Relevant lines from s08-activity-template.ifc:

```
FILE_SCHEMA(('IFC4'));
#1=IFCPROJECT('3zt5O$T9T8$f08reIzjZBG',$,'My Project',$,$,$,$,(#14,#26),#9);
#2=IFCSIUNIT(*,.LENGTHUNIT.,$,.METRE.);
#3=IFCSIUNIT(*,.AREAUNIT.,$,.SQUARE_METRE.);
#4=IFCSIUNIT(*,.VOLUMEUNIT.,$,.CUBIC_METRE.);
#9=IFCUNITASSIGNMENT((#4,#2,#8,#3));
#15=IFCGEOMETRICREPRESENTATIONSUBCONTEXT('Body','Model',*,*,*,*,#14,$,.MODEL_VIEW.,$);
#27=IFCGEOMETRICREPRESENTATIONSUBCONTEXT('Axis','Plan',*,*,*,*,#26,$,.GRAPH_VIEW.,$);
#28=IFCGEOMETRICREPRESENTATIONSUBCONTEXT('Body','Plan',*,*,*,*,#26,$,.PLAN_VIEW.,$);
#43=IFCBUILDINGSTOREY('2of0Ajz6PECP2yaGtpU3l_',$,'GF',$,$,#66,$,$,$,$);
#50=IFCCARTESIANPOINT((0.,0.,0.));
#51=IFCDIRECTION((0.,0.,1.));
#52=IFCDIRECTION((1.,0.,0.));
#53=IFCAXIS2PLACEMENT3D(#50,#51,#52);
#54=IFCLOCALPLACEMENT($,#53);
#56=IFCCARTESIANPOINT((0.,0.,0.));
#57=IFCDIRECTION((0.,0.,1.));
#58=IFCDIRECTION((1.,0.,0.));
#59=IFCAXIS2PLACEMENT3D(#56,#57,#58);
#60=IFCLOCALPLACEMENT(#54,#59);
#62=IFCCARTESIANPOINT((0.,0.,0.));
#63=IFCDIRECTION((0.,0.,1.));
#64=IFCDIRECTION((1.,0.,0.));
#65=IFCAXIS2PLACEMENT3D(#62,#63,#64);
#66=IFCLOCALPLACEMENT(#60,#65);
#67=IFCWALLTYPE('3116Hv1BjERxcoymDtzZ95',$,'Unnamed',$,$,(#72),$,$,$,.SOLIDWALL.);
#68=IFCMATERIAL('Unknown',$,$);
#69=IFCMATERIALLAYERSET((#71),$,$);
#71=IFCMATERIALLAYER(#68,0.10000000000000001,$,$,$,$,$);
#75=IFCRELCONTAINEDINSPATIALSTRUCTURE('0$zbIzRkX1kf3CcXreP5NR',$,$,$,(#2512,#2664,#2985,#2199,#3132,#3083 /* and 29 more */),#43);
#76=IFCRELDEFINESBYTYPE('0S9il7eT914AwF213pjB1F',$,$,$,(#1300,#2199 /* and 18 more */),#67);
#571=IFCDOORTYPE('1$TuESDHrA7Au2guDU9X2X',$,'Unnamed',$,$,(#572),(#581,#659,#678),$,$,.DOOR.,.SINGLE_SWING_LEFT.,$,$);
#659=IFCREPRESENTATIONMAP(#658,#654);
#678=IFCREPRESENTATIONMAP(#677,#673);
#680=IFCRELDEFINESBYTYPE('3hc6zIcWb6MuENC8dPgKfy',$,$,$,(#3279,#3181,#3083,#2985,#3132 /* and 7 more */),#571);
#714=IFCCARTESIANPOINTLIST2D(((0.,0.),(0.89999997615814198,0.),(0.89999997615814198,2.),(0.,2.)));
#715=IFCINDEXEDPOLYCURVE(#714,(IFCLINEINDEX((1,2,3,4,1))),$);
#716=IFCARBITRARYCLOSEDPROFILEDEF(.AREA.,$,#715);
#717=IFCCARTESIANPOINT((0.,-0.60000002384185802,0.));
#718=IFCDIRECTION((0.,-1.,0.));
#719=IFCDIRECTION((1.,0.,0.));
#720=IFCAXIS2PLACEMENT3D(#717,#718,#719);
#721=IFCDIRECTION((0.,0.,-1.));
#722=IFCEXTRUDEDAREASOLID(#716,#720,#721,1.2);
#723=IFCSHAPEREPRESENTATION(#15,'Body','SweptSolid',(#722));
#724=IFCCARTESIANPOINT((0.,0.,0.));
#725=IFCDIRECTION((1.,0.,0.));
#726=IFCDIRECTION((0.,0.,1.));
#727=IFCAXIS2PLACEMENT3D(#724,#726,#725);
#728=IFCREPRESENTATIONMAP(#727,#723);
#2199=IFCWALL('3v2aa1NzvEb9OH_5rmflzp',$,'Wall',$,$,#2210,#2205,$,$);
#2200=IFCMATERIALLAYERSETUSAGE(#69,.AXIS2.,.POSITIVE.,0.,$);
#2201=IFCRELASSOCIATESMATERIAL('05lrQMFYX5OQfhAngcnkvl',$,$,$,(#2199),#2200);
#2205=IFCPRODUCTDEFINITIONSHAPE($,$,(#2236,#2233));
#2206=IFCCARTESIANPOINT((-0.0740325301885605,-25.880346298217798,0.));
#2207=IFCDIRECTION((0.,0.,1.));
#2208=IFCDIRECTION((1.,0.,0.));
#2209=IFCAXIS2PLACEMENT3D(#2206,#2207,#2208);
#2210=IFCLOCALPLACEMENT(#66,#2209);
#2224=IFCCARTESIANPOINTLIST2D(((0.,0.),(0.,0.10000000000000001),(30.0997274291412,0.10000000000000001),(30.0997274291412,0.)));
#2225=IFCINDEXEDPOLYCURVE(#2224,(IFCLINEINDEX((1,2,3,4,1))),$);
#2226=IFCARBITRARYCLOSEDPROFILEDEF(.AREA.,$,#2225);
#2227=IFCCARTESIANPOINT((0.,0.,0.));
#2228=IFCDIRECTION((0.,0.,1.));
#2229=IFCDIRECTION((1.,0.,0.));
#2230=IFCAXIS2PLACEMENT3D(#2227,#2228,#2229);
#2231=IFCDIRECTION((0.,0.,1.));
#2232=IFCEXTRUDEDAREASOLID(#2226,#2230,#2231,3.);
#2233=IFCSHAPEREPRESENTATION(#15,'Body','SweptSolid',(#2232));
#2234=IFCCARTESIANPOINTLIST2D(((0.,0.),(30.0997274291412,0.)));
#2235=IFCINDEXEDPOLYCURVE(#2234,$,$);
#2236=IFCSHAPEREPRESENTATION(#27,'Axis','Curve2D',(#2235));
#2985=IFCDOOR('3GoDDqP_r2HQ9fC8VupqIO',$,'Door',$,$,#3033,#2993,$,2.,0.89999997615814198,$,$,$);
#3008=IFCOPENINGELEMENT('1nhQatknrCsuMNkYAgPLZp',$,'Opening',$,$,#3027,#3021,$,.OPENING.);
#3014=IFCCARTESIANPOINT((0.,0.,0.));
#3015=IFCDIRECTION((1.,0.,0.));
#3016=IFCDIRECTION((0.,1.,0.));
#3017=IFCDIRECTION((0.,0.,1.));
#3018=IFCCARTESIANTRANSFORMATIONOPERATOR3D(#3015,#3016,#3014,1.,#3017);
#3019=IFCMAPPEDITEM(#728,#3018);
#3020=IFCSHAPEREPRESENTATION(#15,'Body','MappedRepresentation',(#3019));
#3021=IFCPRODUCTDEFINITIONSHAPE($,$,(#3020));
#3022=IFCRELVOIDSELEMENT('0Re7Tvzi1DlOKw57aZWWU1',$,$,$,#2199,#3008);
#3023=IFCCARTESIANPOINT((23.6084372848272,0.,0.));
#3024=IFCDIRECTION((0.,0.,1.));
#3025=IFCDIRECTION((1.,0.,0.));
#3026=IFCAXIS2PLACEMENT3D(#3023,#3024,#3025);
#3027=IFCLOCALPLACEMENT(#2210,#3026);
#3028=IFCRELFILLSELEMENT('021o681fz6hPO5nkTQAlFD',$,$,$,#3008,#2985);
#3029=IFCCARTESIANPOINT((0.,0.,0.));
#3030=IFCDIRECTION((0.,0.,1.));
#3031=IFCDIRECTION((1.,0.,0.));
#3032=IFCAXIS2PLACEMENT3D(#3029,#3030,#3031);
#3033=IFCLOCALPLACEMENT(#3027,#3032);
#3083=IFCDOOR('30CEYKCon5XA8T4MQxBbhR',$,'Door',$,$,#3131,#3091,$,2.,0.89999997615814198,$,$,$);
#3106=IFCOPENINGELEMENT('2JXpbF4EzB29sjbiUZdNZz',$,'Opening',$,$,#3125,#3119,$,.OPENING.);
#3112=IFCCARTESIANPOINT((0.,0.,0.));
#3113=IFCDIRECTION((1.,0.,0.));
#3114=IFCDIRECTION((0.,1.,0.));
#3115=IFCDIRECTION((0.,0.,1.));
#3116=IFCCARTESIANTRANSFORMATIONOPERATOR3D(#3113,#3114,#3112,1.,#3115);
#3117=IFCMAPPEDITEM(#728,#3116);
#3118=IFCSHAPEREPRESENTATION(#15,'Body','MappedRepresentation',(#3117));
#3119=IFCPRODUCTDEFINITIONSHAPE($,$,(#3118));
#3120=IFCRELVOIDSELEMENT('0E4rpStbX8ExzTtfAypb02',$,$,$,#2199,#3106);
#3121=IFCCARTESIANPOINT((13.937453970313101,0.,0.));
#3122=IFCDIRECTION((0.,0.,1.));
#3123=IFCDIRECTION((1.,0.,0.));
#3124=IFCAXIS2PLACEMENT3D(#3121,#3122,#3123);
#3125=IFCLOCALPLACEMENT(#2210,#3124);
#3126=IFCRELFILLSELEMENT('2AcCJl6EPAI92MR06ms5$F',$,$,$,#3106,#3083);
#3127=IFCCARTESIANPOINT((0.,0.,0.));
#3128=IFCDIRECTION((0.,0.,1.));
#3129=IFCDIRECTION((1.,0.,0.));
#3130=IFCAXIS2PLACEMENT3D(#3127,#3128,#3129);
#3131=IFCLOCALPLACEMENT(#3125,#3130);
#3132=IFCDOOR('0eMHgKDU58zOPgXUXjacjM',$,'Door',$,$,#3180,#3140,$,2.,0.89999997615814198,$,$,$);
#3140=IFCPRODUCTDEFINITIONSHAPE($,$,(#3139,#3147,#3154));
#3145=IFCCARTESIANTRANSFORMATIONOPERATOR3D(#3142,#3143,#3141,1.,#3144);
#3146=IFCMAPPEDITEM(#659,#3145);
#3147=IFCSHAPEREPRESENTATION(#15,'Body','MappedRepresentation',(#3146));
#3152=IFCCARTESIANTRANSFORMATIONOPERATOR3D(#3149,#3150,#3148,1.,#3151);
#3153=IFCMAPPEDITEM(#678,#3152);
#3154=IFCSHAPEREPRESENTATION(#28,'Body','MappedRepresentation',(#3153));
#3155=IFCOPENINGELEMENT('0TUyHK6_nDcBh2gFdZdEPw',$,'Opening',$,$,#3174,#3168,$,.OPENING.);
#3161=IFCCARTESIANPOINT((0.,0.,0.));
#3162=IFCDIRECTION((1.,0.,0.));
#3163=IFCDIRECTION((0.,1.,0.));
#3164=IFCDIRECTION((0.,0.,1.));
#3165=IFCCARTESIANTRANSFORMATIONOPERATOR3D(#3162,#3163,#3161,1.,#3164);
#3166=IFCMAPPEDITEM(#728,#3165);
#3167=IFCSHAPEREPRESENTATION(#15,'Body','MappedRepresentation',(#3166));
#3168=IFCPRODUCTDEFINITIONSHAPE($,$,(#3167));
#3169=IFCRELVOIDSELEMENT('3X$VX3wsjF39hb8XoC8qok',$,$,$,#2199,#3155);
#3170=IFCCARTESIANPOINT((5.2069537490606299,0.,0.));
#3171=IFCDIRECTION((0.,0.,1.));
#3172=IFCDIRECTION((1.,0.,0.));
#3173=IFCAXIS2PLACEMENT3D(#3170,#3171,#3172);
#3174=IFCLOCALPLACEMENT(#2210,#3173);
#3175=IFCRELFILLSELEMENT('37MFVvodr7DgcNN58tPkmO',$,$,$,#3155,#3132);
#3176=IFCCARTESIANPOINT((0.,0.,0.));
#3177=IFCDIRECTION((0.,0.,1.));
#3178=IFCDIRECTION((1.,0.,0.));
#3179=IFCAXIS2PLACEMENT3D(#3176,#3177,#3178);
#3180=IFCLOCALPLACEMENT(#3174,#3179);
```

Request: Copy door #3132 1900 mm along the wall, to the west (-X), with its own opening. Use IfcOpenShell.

```python
import ifcopenshell
import ifcopenshell.api.feature
import ifcopenshell.api.geometry
import ifcopenshell.api.root
import ifcopenshell.geom
import ifcopenshell.util.element
import ifcopenshell.util.placement
import ifcopenshell.util.shape
import ifcopenshell.util.unit

model = ifcopenshell.open("s08-activity-template.ifc")
unit_scale = ifcopenshell.util.unit.calculate_unit_scale(model)
settings = ifcopenshell.geom.settings()


def volume(element):
    """Net volume in cubic metres, openings subtracted."""
    shape = ifcopenshell.geom.create_shape(settings, element)
    return ifcopenshell.util.shape.get_volume(shape.geometry)


door = model.by_guid("0eMHgKDU58zOPgXUXjacjM")
opening = door.FillsVoids[0].RelatingOpeningElement
wall = opening.VoidsElements[0].RelatingBuildingElement
before = volume(wall)
shift = ifcopenshell.util.placement.get_local_placement(wall.ObjectPlacement)[:3, 0] * -1.9 / unit_scale

# copy_class copies the void relationship, type, container and properties, but no geometry.
new_opening = ifcopenshell.api.root.copy_class(model, product=opening)
new_opening.Representation = ifcopenshell.util.element.copy_deep(
    model, opening.Representation, exclude=["IfcGeometricRepresentationContext", "IfcRepresentationMap"]
)
new_door = ifcopenshell.api.root.copy_class(model, product=door)
new_door.Representation = ifcopenshell.util.element.copy_deep(
    model, door.Representation, exclude=["IfcGeometricRepresentationContext", "IfcRepresentationMap"]
)
ifcopenshell.api.feature.add_filling(model, opening=new_opening, element=new_door)

for old, new in ((opening, new_opening), (door, new_door)):
    matrix = ifcopenshell.util.placement.get_local_placement(old.ObjectPlacement)
    matrix[:3, 3] += shift
    ifcopenshell.api.geometry.edit_object_placement(model, product=new, matrix=matrix, is_si=False)

after = volume(wall)

print(f"wall volume {before:.3f} -> {after:.3f} m3")

model.write("s08-activity-template_rev.ifc")
```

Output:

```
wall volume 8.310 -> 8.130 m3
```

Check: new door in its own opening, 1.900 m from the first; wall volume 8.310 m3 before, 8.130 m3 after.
